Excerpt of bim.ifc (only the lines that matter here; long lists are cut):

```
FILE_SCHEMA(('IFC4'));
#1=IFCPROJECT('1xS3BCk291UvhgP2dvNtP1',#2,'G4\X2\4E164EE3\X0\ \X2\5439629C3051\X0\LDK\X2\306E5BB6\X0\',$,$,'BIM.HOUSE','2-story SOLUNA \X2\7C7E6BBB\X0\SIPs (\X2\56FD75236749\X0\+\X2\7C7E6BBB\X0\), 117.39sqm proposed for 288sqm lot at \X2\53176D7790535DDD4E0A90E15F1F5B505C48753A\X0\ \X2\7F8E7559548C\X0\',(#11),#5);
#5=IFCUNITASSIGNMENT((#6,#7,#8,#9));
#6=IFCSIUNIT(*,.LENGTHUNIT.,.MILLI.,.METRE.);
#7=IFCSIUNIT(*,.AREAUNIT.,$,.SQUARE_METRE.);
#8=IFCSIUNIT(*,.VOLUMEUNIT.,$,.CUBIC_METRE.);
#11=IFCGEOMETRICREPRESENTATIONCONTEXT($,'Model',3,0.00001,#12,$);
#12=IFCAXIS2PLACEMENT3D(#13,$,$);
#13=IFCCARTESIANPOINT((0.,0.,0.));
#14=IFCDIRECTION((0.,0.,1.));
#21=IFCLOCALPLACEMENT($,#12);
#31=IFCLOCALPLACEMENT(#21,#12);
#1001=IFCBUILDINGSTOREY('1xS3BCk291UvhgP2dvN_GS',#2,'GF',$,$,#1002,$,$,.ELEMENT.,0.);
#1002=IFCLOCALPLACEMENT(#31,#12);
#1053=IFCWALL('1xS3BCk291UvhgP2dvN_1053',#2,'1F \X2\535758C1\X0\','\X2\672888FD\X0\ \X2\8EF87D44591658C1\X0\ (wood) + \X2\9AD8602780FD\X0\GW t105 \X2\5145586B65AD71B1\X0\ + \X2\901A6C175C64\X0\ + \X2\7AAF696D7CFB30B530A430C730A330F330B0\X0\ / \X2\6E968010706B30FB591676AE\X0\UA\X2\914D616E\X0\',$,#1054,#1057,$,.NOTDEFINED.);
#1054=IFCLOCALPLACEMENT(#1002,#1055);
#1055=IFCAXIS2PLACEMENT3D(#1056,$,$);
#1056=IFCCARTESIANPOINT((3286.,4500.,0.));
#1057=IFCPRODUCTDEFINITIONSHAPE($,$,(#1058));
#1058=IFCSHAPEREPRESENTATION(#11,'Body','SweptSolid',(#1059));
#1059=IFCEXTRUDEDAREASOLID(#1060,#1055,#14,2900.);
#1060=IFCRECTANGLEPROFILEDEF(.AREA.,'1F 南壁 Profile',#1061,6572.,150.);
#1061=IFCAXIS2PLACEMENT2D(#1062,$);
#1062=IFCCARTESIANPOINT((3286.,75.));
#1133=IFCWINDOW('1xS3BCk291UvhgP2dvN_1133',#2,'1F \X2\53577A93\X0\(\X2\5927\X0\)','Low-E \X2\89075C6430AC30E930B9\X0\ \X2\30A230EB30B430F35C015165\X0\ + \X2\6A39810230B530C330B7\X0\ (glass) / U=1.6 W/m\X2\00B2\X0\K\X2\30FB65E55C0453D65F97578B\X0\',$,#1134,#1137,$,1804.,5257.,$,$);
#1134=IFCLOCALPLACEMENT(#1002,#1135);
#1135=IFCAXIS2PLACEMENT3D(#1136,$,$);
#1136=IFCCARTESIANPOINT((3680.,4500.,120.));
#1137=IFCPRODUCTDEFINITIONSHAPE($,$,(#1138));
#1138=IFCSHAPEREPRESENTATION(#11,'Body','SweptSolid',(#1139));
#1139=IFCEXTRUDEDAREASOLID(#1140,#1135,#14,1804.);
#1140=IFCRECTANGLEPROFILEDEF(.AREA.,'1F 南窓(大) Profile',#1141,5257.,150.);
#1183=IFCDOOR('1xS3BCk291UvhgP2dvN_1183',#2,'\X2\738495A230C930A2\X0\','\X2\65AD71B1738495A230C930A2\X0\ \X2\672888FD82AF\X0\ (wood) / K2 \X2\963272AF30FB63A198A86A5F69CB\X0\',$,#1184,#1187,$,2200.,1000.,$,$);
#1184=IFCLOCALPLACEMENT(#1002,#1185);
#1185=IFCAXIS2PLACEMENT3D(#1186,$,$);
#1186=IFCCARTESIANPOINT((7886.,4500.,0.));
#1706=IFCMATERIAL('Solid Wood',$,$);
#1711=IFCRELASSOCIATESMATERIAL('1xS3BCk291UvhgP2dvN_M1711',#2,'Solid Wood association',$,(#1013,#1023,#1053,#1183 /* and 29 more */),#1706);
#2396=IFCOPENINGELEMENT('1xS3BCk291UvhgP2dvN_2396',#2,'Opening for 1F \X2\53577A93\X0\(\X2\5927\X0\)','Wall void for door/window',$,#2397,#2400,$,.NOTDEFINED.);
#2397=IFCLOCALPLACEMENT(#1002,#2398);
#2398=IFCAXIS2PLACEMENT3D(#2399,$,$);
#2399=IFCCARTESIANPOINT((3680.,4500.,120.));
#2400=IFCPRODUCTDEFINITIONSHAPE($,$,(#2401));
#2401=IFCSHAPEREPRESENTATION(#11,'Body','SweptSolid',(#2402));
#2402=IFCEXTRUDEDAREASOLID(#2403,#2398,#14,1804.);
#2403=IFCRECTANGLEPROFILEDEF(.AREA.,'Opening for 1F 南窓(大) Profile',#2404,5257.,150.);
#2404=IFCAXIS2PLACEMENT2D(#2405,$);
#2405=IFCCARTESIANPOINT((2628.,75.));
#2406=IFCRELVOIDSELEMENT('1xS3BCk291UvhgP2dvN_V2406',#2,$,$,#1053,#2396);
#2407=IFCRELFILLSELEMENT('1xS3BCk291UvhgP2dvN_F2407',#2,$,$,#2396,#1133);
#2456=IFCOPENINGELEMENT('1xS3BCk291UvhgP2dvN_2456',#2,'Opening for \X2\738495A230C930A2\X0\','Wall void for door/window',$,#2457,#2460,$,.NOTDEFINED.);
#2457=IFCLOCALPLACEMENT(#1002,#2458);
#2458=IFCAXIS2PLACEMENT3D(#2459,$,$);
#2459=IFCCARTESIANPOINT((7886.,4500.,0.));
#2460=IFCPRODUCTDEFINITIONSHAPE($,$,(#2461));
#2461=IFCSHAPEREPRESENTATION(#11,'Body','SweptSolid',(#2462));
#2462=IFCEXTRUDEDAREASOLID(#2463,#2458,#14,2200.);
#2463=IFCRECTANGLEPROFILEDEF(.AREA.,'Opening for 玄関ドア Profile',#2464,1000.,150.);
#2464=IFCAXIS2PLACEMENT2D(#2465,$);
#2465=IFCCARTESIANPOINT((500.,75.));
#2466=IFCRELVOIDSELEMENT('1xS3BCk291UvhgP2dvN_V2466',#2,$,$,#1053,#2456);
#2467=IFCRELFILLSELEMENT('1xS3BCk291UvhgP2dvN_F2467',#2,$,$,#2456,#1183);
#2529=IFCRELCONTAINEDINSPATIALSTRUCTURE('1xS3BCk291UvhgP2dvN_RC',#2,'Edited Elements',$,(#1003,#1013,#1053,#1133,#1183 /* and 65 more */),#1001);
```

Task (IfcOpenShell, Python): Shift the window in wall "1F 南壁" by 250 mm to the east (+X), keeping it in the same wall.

```python
import ifcopenshell
import ifcopenshell.api.geometry
import ifcopenshell.util.placement

model = ifcopenshell.open("bim.ifc")

window = model.by_id(1133)
opening = window.FillsVoids[0].RelatingOpeningElement
wall = opening.VoidsElements[0].RelatingBuildingElement

wall_matrix = ifcopenshell.util.placement.get_local_placement(wall.ObjectPlacement)
shift = wall_matrix[:3, 0] * 250.0
before = ifcopenshell.util.placement.get_local_placement(window.ObjectPlacement)[:3, 3].copy()

# The window is not placed relative to its opening, so move both.
for product in (opening, window):
    matrix = ifcopenshell.util.placement.get_local_placement(product.ObjectPlacement)
    matrix[:3, 3] += shift
    ifcopenshell.api.geometry.edit_object_placement(model, product=product, matrix=matrix, is_si=False)

after = ifcopenshell.util.placement.get_local_placement(window.ObjectPlacement)[:3, 3]
print("window moved by", (after - before).round(3) + 0.0)

model.write("bim_edited.ifc")
```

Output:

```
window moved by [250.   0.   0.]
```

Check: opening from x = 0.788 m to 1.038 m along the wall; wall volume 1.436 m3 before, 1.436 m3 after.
